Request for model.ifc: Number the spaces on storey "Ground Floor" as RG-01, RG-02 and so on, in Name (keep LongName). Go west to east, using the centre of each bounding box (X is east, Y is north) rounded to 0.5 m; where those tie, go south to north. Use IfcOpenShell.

First a look at what the model holds.

```python
import ifcopenshell
import ifcopenshell.util.element
import ifcopenshell.util.placement

model = ifcopenshell.open("model.ifc")
print(model.schema)
storey = next(s for s in model.by_type("IfcBuildingStorey") if s.Name == "Ground Floor")
spaces = [e for e in ifcopenshell.util.element.get_decomposition(storey) if e.is_a("IfcSpace")]
for e in sorted(spaces, key=lambda e: e.id()):
    origin = ifcopenshell.util.placement.get_local_placement(e.ObjectPlacement)[:3, 3]
    print(e.id(), e.Name, e.LongName, origin.round(2) + 0.0, sep=" | ")
```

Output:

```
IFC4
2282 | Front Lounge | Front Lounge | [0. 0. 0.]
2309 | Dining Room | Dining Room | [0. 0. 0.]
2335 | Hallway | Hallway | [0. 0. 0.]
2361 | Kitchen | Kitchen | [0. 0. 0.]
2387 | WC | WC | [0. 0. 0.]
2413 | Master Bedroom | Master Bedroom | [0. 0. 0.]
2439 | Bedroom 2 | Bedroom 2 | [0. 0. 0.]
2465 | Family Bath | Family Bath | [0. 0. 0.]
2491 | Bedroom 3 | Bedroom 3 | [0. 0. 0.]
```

```python
import ifcopenshell
import ifcopenshell.geom
import ifcopenshell.util.element
import ifcopenshell.util.shape

model = ifcopenshell.open("model.ifc")
settings = ifcopenshell.geom.settings()
settings.set("use-world-coords", True)


def centre(element):
    shape = ifcopenshell.geom.create_shape(settings, element)
    return ifcopenshell.util.shape.get_bbox_centroid(shape.geometry)


storey = next(s for s in model.by_type("IfcBuildingStorey") if s.Name == "Ground Floor")
spaces = [e for e in ifcopenshell.util.element.get_decomposition(storey) if e.is_a("IfcSpace")]

# Insertion points can sit at a corner or the storey origin, so sort by the geometry (in metres).
centres = {e: centre(e) for e in spaces}
spaces.sort(key=lambda e: (round(centres[e][0] / 0.5), centres[e][1]))

for i, e in enumerate(spaces, start=1):
    number = f"RG-{i:02d}"
    e.Name = number
    print(e.id(), number)

model.write("model_updated.ifc")
```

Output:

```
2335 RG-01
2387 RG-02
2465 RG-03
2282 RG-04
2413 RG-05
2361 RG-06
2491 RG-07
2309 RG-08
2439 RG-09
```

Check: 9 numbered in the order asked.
